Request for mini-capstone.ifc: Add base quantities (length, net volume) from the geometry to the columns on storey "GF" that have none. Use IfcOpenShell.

First a look at what the model holds.

```python
import ifcopenshell
import ifcopenshell.util.element
import ifcopenshell.util.unit

model = ifcopenshell.open("mini-capstone.ifc")
print(model.schema)
for unit_type in ("LENGTHUNIT", "AREAUNIT", "VOLUMEUNIT"):
    print(unit_type, ifcopenshell.util.unit.calculate_unit_scale(model, unit_type))
storey = next(s for s in model.by_type("IfcBuildingStorey") if s.Name == "GF")
columns = [e for e in ifcopenshell.util.element.get_decomposition(storey) if e.is_a("IfcColumn")]
for e in sorted(columns, key=lambda e: e.id()):
    print(e.id(), e.is_a(), e.Name, list(ifcopenshell.util.element.get_psets(e, qtos_only=True)), sep=" | ")
```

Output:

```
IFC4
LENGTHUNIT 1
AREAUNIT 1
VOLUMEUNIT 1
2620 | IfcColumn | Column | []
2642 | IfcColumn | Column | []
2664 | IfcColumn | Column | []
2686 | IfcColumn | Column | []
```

```python
import ifcopenshell
import ifcopenshell.api.pset
import ifcopenshell.geom
import ifcopenshell.util.element
import ifcopenshell.util.shape
import ifcopenshell.util.unit

model = ifcopenshell.open("mini-capstone.ifc")
unit_scale = ifcopenshell.util.unit.calculate_unit_scale(model)
volume_scale = ifcopenshell.util.unit.calculate_unit_scale(model, "VOLUMEUNIT")
settings = ifcopenshell.geom.settings()

storey = next(s for s in model.by_type("IfcBuildingStorey") if s.Name == "GF")
columns = [e for e in ifcopenshell.util.element.get_decomposition(storey) if e.is_a("IfcColumn")]

for e in sorted(columns, key=lambda e: e.id()):
    if ifcopenshell.util.element.get_psets(e, qtos_only=True, should_inherit=False):
        continue
    # Geometry comes back in metres, in the element's own axes.
    shape = ifcopenshell.geom.create_shape(settings, e)
    values = {
        "Length": ifcopenshell.util.shape.get_z(shape.geometry) / unit_scale,
        "NetVolume": ifcopenshell.util.shape.get_volume(shape.geometry) / volume_scale,
    }
    qto = ifcopenshell.api.pset.add_qto(model, product=e, name="Qto_ColumnBaseQuantities")
    ifcopenshell.api.pset.edit_qto(model, qto=qto, properties=values)
    print(e.id(), {k: round(v, 3) for k, v in values.items()})

model.write("mini-capstone_rev.ifc")
```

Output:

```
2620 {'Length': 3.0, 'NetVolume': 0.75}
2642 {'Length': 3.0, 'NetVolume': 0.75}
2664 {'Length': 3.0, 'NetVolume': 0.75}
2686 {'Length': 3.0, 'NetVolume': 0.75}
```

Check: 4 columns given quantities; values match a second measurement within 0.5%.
